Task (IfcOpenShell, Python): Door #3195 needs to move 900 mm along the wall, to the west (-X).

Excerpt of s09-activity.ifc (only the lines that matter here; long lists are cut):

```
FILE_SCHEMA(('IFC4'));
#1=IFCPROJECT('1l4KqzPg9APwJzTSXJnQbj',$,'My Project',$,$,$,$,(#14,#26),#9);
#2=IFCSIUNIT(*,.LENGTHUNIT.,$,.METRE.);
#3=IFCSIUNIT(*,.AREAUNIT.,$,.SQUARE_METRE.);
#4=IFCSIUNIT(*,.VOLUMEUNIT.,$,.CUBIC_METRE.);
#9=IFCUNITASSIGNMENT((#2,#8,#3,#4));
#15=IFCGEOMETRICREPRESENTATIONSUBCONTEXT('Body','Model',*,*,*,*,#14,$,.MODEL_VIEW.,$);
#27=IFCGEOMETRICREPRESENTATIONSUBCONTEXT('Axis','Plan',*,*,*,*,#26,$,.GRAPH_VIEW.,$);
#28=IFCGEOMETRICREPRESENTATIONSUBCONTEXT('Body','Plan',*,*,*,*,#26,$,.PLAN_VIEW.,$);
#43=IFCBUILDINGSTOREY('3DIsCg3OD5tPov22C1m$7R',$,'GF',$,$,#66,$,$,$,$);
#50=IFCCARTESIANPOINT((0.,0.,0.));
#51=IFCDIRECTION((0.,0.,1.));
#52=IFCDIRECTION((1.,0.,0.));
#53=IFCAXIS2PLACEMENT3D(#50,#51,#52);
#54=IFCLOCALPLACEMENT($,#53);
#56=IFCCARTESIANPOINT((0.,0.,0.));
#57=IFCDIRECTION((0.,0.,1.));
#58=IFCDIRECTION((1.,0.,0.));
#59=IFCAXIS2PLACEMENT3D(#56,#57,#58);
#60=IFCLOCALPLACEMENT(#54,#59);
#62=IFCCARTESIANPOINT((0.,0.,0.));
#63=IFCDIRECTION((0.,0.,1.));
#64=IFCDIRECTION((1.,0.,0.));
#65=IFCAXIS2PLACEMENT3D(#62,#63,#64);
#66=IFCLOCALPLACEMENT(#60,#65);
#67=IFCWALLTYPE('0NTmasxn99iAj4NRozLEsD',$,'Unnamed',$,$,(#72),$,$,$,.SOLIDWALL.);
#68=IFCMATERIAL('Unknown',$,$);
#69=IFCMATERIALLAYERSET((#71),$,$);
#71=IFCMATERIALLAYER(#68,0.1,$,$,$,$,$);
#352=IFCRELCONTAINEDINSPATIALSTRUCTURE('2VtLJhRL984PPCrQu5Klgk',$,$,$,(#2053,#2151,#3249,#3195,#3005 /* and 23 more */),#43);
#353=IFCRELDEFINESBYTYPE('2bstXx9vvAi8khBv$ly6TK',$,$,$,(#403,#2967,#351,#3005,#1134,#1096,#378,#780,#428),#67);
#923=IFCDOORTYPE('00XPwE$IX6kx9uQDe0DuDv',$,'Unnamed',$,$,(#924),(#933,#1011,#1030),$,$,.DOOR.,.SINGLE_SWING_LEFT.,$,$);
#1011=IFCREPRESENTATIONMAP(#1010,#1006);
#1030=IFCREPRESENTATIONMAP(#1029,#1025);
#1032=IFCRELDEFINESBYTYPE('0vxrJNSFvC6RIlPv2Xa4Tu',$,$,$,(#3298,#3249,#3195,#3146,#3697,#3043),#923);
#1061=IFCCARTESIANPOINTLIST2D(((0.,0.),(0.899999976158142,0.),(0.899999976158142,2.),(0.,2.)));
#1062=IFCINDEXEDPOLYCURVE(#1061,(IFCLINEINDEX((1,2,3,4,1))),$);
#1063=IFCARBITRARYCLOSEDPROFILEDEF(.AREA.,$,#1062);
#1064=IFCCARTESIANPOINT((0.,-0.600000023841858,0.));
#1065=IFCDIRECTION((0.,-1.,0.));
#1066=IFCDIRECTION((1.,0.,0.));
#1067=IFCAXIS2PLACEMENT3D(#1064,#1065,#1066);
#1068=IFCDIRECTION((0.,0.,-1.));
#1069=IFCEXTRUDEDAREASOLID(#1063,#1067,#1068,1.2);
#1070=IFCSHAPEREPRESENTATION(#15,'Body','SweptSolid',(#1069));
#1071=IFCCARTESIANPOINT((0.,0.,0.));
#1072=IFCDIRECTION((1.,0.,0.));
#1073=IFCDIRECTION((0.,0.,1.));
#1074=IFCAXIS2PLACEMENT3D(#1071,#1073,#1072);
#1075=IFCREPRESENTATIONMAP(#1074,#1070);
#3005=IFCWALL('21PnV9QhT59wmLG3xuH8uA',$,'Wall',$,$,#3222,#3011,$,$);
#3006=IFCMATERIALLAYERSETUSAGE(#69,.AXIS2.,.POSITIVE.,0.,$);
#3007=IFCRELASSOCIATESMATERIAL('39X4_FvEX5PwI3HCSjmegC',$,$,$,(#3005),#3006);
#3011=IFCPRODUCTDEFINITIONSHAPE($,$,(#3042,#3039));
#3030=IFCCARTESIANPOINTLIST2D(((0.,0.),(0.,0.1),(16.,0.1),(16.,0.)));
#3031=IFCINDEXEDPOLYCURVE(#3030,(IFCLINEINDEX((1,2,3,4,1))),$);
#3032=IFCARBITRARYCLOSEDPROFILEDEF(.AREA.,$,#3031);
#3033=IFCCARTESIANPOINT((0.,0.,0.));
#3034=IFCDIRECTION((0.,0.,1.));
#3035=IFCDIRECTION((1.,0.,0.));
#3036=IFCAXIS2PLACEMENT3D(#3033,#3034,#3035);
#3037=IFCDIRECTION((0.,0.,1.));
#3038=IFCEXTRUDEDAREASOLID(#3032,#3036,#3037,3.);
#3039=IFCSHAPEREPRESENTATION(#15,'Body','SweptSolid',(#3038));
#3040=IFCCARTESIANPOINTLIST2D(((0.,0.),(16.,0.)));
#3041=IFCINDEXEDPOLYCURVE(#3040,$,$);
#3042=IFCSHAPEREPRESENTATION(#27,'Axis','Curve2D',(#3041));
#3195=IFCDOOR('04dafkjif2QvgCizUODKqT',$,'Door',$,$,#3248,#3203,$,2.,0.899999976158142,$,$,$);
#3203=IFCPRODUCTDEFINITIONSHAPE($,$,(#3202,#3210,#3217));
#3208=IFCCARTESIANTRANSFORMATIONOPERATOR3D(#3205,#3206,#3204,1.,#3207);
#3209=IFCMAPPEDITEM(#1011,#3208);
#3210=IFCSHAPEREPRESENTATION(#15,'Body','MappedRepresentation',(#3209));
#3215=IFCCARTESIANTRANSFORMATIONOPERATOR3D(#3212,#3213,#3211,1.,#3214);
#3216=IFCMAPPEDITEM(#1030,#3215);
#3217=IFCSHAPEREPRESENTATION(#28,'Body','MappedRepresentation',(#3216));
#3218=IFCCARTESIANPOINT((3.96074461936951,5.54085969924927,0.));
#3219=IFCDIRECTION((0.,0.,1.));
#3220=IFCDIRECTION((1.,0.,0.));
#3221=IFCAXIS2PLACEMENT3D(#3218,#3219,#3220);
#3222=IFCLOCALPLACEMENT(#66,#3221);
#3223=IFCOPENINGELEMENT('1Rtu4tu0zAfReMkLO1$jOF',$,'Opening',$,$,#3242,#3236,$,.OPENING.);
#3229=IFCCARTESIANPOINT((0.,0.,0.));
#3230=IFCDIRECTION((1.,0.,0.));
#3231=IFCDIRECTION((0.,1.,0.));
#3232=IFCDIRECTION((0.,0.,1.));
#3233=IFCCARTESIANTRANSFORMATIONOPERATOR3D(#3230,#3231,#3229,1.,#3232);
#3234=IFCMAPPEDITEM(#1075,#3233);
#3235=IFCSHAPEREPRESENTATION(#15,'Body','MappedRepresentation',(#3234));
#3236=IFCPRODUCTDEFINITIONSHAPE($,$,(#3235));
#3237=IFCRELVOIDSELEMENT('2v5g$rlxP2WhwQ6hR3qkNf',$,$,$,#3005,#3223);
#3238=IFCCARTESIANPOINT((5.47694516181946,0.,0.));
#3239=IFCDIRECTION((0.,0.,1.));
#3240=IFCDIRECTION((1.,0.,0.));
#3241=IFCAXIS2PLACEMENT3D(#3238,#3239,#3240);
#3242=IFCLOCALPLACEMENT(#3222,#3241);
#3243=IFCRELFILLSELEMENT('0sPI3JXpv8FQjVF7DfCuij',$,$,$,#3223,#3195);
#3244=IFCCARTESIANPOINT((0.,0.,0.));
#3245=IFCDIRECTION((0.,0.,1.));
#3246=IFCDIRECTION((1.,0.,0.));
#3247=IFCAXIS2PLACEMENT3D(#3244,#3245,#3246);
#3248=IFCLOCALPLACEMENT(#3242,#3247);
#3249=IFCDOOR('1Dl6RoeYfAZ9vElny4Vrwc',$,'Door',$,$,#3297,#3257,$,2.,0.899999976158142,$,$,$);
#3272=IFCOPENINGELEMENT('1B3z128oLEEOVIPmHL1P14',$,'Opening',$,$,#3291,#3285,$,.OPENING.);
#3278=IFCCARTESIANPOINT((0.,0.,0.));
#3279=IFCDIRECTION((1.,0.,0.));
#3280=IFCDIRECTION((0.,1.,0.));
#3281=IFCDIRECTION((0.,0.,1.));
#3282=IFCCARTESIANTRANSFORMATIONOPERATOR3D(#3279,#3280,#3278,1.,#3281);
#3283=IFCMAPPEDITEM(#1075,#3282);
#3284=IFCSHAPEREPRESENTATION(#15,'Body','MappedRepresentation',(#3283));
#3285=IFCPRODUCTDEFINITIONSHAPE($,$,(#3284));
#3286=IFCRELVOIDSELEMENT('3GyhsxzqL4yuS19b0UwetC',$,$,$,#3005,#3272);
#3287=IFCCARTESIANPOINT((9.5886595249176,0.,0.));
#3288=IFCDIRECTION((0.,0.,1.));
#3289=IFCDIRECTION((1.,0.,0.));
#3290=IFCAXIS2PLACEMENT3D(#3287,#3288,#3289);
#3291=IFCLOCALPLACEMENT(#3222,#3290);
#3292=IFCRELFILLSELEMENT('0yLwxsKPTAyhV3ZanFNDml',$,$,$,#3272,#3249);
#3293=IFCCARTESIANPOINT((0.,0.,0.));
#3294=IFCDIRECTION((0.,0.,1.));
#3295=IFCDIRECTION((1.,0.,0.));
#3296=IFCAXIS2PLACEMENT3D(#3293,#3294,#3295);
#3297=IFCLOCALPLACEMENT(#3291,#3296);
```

```python
import ifcopenshell
import ifcopenshell.api.geometry
import ifcopenshell.util.placement

model = ifcopenshell.open("s09-activity.ifc")

door = model.by_guid("04dafkjif2QvgCizUODKqT")
opening = door.FillsVoids[0].RelatingOpeningElement
wall = opening.VoidsElements[0].RelatingBuildingElement

wall_matrix = ifcopenshell.util.placement.get_local_placement(wall.ObjectPlacement)
shift = wall_matrix[:3, 0] * -0.9
before = ifcopenshell.util.placement.get_local_placement(door.ObjectPlacement)[:3, 3].copy()

# The door is placed relative to its opening, so it follows when the opening moves.
matrix = ifcopenshell.util.placement.get_local_placement(opening.ObjectPlacement)
matrix[:3, 3] += shift
ifcopenshell.api.geometry.edit_object_placement(
    model, product=opening, matrix=matrix, is_si=False, should_transform_children=True
)

after = ifcopenshell.util.placement.get_local_placement(door.ObjectPlacement)[:3, 3]
print("door moved by", (after - before).round(3) + 0.0)

model.write("s09-activity_v2.ifc")
```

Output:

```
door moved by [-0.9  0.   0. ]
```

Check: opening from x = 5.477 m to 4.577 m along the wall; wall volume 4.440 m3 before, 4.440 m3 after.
